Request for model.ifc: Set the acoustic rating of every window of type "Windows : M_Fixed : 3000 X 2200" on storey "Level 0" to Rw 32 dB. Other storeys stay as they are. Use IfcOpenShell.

First a look at what the model holds.

```python
import ifcopenshell
import ifcopenshell.util.element

model = ifcopenshell.open("model.ifc")
print(model.schema)
storey = next(s for s in model.by_type("IfcBuildingStorey") if s.Name == "Level 0")
windows = [e for e in ifcopenshell.util.element.get_decomposition(storey) if e.is_a("IfcWindow")]
seen = {}
for e in windows:
    element_type = ifcopenshell.util.element.get_type(e)
    key = (element_type.Name if element_type != e and element_type else None, ifcopenshell.util.element.get_pset(e, "Pset_WindowCommon", "AcousticRating"))
    seen[key] = seen.get(key, 0) + 1
for (name, value), count in sorted(seen.items(), key=str):
    print(count, "x", name, "|", value)
```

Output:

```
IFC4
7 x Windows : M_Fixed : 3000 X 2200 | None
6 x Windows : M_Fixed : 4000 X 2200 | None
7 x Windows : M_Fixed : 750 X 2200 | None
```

```python
import ifcopenshell
import ifcopenshell.api.pset
import ifcopenshell.util.element

model = ifcopenshell.open("model.ifc")

storey = next(s for s in model.by_type("IfcBuildingStorey") if s.Name == "Level 0")
windows = [e for e in ifcopenshell.util.element.get_decomposition(storey) if e.is_a("IfcWindow")]

count = 0
for e in windows:
    element_type = ifcopenshell.util.element.get_type(e)
    if element_type in (None, e) or element_type.Name != "Windows : M_Fixed : 3000 X 2200":
        continue
    # add_pset returns the element's existing set when there is one.
    pset = ifcopenshell.api.pset.add_pset(model, product=e, name="Pset_WindowCommon")
    ifcopenshell.api.pset.edit_pset(model, pset=pset, properties={"AcousticRating": "Rw 32 dB"})
    count += 1

print(count, "windows updated")

model.write("model-out.ifc")
```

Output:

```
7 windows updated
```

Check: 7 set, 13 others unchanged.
